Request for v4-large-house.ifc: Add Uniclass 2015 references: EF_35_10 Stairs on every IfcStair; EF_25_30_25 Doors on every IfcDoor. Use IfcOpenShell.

First a look at what the model holds.

```python
import ifcopenshell

model = ifcopenshell.open("v4-large-house.ifc")
print(model.schema)
print("classifications:", [c.Name for c in model.by_type("IfcClassification")])
for ifc_class in ("IfcDoor", "IfcRoof", "IfcStair", "IfcWall", "IfcWindow"):
    print(ifc_class, len(model.by_type(ifc_class)))
```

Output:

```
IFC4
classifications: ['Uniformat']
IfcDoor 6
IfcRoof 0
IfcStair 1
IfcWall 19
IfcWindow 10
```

```python
import ifcopenshell
import ifcopenshell.api.classification

model = ifcopenshell.open("v4-large-house.ifc")

system = ifcopenshell.api.classification.add_classification(model, classification="Uniclass 2015")

codes = {
    "IfcStair": ("EF_35_10", "Stairs"),
    "IfcDoor": ("EF_25_30_25", "Doors"),
}
for ifc_class, (code, name) in codes.items():
    products = model.by_type(ifc_class)
    ifcopenshell.api.classification.add_reference(
        model, products=products, classification=system, identification=code, name=name
    )
    print(code, len(products))

model.write("v4-large-house_rev.ifc")
```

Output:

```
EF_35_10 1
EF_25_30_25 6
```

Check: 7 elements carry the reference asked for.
